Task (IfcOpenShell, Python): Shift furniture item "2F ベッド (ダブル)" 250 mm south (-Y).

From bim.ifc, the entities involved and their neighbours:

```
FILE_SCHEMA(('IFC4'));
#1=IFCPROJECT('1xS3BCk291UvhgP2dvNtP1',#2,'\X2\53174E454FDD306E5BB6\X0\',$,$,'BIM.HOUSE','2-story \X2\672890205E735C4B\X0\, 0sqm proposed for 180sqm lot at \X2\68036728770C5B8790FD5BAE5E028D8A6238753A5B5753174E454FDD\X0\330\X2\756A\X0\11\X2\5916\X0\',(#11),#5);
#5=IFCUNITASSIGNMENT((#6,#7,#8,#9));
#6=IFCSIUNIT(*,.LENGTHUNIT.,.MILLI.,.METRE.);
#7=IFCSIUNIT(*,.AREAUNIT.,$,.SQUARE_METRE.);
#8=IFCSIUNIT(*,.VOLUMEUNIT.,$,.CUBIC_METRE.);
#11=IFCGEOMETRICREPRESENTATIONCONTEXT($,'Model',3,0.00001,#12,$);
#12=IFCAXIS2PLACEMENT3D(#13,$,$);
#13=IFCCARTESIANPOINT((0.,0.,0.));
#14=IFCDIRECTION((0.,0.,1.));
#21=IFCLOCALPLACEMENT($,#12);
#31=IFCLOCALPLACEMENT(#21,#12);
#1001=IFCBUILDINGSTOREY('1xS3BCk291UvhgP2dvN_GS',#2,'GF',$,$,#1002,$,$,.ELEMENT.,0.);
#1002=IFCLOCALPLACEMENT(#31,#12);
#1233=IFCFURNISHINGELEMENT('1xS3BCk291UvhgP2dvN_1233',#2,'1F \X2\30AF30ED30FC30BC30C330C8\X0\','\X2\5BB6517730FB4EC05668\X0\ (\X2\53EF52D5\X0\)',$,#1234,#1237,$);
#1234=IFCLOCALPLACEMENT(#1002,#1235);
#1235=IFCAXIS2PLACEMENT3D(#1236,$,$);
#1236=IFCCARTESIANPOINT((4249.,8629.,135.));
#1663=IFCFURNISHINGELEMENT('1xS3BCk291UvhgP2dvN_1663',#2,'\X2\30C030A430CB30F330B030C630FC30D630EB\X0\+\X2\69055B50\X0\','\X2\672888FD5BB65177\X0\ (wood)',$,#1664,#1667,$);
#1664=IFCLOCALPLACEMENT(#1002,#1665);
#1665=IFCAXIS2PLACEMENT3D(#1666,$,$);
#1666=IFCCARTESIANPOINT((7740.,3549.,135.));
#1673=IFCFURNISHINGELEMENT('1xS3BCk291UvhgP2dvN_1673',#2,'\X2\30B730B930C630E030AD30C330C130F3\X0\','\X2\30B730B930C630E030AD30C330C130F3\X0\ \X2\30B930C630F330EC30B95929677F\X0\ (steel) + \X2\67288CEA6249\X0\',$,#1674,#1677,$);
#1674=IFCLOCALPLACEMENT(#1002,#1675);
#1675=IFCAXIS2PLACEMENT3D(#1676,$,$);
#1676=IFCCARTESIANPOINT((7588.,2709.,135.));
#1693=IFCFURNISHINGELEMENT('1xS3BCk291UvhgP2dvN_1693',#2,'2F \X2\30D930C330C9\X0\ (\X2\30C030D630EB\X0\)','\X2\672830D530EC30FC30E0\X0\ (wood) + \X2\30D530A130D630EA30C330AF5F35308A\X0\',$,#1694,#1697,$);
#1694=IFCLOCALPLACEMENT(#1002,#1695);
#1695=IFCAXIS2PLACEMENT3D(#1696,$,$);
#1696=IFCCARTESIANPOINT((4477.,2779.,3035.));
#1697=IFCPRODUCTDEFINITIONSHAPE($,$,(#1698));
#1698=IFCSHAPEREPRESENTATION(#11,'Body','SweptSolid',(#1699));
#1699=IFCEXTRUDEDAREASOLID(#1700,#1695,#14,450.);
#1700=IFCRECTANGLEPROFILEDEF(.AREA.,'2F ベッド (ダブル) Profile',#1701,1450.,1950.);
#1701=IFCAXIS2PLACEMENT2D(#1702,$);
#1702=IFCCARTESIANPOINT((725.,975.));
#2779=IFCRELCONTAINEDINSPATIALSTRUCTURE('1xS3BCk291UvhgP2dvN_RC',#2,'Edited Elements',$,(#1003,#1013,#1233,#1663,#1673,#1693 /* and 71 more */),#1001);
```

```python
import ifcopenshell
import ifcopenshell.api.geometry
import ifcopenshell.util.placement

model = ifcopenshell.open("bim.ifc")

item = model.by_guid("1xS3BCk291UvhgP2dvN_1693")
matrix = ifcopenshell.util.placement.get_local_placement(item.ObjectPlacement)
matrix[1, 3] -= 250.0
ifcopenshell.api.geometry.edit_object_placement(model, product=item, matrix=matrix, is_si=False)

print(ifcopenshell.util.placement.get_local_placement(item.ObjectPlacement).round(3) + 0.0)

model.write("bim_edited.ifc")
```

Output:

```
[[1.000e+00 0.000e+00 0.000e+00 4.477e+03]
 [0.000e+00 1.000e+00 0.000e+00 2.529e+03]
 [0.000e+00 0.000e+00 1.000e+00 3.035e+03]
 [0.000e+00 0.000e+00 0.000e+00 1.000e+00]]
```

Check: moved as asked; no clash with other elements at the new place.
